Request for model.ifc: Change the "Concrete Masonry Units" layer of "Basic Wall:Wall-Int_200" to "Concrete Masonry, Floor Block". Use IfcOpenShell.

First a look at what the model holds.

```python
import ifcopenshell
import ifcopenshell.util.element

model = ifcopenshell.open("model.ifc")
print(model.schema)
for layer_set in model.by_type("IfcMaterialLayerSet"):
    if layer_set.LayerSetName == "Basic Wall:Wall-Int_200":
        for layer in layer_set.MaterialLayers:
            print(layer.id(), layer.Material and layer.Material.Name, layer.LayerThickness, sep=" | ")
        print(len(ifcopenshell.util.element.get_elements_by_material(model, layer_set)), "elements and types use it")
print(sorted(m.Name for m in model.by_type("IfcMaterial") if m.Name)[:60])
```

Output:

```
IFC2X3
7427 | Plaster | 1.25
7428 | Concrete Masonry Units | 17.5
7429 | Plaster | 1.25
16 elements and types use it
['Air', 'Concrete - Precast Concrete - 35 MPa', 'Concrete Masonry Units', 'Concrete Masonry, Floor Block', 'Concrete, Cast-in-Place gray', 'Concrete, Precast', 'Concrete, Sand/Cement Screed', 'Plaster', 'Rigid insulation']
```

```python
import ifcopenshell
import ifcopenshell.api.material

model = ifcopenshell.open("model.ifc")

layer_set = next(s for s in model.by_type("IfcMaterialLayerSet") if s.LayerSetName == "Basic Wall:Wall-Int_200")
layer = next(l for l in layer_set.MaterialLayers if l.Material and l.Material.Name == "Concrete Masonry Units")
material = next(m for m in model.by_type("IfcMaterial") if m.Name == "Concrete Masonry, Floor Block")

# Point this one layer at the other material; renaming the old one would change it everywhere.
ifcopenshell.api.material.edit_layer(model, layer=layer, attributes={}, material=material)

print([l.Material.Name if l.Material else None for l in layer_set.MaterialLayers])

model.write("model_updated.ifc")
```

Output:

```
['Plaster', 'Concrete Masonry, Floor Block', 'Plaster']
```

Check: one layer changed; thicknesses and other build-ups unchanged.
